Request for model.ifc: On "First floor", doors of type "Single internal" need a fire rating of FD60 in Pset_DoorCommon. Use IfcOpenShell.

First a look at what the model holds.

```python
import ifcopenshell
import ifcopenshell.util.element

model = ifcopenshell.open("model.ifc")
print(model.schema)
storey = next(s for s in model.by_type("IfcBuildingStorey") if s.Name == "First floor")
doors = [e for e in ifcopenshell.util.element.get_decomposition(storey) if e.is_a("IfcDoor")]
seen = {}
for e in doors:
    element_type = ifcopenshell.util.element.get_type(e)
    key = (element_type.Name if element_type != e and element_type else None, ifcopenshell.util.element.get_pset(e, "Pset_DoorCommon", "FireRating"))
    seen[key] = seen.get(key, 0) + 1
for (name, value), count in sorted(seen.items(), key=str):
    print(count, "x", name, "|", value)
```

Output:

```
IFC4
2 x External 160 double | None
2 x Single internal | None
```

```python
import ifcopenshell
import ifcopenshell.api.pset
import ifcopenshell.util.element

model = ifcopenshell.open("model.ifc")

storey = next(s for s in model.by_type("IfcBuildingStorey") if s.Name == "First floor")
doors = [e for e in ifcopenshell.util.element.get_decomposition(storey) if e.is_a("IfcDoor")]

count = 0
for e in doors:
    element_type = ifcopenshell.util.element.get_type(e)
    if element_type in (None, e) or element_type.Name != "Single internal":
        continue
    # add_pset returns the element's existing set when there is one.
    pset = ifcopenshell.api.pset.add_pset(model, product=e, name="Pset_DoorCommon")
    ifcopenshell.api.pset.edit_pset(model, pset=pset, properties={"FireRating": "FD60"})
    count += 1

print(count, "doors updated")

model.write("model-out.ifc")
```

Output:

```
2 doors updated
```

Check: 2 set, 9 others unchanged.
